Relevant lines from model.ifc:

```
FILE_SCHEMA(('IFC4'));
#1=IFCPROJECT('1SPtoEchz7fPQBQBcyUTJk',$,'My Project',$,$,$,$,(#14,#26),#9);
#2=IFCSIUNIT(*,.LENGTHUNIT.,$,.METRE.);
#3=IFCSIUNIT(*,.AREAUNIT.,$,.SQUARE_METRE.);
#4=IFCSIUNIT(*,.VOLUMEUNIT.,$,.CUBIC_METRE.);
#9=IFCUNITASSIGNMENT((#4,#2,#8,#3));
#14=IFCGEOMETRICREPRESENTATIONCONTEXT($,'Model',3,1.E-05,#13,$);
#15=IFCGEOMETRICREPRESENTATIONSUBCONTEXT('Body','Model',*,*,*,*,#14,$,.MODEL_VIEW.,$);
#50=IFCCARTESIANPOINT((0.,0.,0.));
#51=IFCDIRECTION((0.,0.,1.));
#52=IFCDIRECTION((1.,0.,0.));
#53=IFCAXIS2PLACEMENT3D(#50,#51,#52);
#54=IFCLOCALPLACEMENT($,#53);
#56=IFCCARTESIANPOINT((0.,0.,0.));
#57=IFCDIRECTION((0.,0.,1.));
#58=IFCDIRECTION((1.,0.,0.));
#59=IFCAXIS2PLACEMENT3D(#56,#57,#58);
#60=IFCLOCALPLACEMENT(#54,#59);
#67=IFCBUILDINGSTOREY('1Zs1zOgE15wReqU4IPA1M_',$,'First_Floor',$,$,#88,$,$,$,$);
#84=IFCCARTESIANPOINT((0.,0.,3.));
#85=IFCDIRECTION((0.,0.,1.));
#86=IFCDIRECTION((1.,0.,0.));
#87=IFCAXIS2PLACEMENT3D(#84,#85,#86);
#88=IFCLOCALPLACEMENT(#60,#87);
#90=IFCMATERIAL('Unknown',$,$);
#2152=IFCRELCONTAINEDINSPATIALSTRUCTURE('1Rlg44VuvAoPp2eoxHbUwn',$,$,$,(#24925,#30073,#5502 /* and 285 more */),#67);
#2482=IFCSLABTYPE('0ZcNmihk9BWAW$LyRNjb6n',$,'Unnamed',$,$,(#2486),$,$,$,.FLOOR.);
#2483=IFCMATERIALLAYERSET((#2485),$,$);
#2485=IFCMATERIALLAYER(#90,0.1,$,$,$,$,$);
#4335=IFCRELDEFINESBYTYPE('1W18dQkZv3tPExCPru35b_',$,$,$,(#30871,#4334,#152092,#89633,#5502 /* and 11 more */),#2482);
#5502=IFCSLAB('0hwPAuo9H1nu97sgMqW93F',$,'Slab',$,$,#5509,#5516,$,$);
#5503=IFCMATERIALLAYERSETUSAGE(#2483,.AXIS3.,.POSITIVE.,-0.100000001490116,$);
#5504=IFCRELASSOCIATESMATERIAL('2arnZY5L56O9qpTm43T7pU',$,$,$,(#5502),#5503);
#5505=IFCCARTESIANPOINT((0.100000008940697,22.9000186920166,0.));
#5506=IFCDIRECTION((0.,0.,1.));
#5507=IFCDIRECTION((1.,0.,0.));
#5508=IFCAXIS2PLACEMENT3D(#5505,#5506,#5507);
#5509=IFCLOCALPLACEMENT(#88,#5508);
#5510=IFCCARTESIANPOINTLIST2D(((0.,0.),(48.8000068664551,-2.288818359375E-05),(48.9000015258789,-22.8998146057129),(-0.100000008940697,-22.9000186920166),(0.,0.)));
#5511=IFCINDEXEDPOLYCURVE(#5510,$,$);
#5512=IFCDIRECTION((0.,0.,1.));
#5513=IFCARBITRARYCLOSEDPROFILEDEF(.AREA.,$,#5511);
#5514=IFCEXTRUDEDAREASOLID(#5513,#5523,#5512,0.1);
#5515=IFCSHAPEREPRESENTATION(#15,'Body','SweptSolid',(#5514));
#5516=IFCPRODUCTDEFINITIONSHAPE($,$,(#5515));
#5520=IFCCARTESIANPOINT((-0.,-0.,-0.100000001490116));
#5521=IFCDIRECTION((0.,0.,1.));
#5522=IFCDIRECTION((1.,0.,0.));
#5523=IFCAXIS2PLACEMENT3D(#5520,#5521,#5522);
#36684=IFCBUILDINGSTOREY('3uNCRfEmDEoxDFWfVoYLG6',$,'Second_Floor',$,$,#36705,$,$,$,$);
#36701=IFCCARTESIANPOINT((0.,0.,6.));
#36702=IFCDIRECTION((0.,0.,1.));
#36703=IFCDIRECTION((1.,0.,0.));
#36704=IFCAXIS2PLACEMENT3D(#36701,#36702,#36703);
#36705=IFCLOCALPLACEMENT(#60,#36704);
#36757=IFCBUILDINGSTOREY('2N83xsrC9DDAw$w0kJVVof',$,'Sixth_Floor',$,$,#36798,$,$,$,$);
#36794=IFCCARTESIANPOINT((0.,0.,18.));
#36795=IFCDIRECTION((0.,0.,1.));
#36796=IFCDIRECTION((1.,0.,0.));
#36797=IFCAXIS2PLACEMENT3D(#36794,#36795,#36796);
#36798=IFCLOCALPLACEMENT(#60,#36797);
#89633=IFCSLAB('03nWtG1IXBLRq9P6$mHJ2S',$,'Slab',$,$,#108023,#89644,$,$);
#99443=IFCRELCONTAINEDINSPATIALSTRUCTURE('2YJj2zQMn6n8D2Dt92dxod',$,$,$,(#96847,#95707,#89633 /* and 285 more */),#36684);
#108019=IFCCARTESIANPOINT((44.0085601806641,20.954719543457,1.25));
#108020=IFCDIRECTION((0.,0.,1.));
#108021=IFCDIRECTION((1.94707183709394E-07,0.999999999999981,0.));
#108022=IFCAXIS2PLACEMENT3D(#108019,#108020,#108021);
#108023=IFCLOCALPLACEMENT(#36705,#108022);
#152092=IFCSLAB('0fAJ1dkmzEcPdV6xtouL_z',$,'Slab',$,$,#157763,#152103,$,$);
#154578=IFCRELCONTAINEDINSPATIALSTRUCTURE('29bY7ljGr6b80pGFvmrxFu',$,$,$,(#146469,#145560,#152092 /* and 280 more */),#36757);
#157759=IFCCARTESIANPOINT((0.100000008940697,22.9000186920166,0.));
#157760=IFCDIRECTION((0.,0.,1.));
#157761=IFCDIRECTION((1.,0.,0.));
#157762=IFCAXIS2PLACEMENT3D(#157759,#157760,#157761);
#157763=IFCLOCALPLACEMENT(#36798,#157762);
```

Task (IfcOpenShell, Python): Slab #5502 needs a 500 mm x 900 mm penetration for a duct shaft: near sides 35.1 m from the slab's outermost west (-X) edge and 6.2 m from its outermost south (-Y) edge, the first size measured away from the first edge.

```python
import numpy as np
import ifcopenshell
import ifcopenshell.api.feature
import ifcopenshell.api.geometry
import ifcopenshell.api.root
import ifcopenshell.geom
import ifcopenshell.util.placement
import ifcopenshell.util.representation
import ifcopenshell.util.shape
import ifcopenshell.util.unit

model = ifcopenshell.open("model.ifc")
unit_scale = ifcopenshell.util.unit.calculate_unit_scale(model)
settings = ifcopenshell.geom.settings()


def volume(element):
    """Net volume in cubic metres, openings subtracted."""
    shape = ifcopenshell.geom.create_shape(settings, element)
    return ifcopenshell.util.shape.get_volume(shape.geometry)


slab = model.by_guid("0hwPAuo9H1nu97sgMqW93F")
before = volume(slab)

# Extent in the slab's own axes, in metres. The edges named are its -X and -Y sides.
slab_shape = ifcopenshell.geom.create_shape(settings, slab)
vertices = ifcopenshell.util.shape.get_vertices(slab_shape.geometry)
x_min, y_min, bottom = vertices.min(axis=0)
top = vertices[:, 2].max()

opening = ifcopenshell.api.root.create_entity(model, ifc_class="IfcOpeningElement", name="Duct shaft opening", predefined_type="OPENING")
context = ifcopenshell.util.representation.get_context(model, "Model", "Body", "MODEL_VIEW")
width, depth = 0.5, 0.9
outline = [(0.0, 0.0), (width, 0.0), (width, depth), (0.0, depth), (0.0, 0.0)]
# Overshoot both faces by 50 mm so the cut is clean.
shape = ifcopenshell.api.geometry.add_slab_representation(
    model, context=context, depth=top - bottom + 0.1, polyline=outline
)
ifcopenshell.api.geometry.assign_representation(model, product=opening, representation=shape)

matrix = ifcopenshell.util.placement.get_local_placement(slab.ObjectPlacement)
matrix[:, 3] = matrix @ np.append(np.array([x_min + 35.1, y_min + 6.2, bottom - 0.05]) / unit_scale, 1.0)
ifcopenshell.api.geometry.edit_object_placement(model, product=opening, matrix=matrix, is_si=False)
ifcopenshell.api.feature.add_feature(model, feature=opening, element=slab)

after = volume(slab)

print(f"slab volume {before:.3f} -> {after:.3f} m3")

model.write("model_v2.ifc")
```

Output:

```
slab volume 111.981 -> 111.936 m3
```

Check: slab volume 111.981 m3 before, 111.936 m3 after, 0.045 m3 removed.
